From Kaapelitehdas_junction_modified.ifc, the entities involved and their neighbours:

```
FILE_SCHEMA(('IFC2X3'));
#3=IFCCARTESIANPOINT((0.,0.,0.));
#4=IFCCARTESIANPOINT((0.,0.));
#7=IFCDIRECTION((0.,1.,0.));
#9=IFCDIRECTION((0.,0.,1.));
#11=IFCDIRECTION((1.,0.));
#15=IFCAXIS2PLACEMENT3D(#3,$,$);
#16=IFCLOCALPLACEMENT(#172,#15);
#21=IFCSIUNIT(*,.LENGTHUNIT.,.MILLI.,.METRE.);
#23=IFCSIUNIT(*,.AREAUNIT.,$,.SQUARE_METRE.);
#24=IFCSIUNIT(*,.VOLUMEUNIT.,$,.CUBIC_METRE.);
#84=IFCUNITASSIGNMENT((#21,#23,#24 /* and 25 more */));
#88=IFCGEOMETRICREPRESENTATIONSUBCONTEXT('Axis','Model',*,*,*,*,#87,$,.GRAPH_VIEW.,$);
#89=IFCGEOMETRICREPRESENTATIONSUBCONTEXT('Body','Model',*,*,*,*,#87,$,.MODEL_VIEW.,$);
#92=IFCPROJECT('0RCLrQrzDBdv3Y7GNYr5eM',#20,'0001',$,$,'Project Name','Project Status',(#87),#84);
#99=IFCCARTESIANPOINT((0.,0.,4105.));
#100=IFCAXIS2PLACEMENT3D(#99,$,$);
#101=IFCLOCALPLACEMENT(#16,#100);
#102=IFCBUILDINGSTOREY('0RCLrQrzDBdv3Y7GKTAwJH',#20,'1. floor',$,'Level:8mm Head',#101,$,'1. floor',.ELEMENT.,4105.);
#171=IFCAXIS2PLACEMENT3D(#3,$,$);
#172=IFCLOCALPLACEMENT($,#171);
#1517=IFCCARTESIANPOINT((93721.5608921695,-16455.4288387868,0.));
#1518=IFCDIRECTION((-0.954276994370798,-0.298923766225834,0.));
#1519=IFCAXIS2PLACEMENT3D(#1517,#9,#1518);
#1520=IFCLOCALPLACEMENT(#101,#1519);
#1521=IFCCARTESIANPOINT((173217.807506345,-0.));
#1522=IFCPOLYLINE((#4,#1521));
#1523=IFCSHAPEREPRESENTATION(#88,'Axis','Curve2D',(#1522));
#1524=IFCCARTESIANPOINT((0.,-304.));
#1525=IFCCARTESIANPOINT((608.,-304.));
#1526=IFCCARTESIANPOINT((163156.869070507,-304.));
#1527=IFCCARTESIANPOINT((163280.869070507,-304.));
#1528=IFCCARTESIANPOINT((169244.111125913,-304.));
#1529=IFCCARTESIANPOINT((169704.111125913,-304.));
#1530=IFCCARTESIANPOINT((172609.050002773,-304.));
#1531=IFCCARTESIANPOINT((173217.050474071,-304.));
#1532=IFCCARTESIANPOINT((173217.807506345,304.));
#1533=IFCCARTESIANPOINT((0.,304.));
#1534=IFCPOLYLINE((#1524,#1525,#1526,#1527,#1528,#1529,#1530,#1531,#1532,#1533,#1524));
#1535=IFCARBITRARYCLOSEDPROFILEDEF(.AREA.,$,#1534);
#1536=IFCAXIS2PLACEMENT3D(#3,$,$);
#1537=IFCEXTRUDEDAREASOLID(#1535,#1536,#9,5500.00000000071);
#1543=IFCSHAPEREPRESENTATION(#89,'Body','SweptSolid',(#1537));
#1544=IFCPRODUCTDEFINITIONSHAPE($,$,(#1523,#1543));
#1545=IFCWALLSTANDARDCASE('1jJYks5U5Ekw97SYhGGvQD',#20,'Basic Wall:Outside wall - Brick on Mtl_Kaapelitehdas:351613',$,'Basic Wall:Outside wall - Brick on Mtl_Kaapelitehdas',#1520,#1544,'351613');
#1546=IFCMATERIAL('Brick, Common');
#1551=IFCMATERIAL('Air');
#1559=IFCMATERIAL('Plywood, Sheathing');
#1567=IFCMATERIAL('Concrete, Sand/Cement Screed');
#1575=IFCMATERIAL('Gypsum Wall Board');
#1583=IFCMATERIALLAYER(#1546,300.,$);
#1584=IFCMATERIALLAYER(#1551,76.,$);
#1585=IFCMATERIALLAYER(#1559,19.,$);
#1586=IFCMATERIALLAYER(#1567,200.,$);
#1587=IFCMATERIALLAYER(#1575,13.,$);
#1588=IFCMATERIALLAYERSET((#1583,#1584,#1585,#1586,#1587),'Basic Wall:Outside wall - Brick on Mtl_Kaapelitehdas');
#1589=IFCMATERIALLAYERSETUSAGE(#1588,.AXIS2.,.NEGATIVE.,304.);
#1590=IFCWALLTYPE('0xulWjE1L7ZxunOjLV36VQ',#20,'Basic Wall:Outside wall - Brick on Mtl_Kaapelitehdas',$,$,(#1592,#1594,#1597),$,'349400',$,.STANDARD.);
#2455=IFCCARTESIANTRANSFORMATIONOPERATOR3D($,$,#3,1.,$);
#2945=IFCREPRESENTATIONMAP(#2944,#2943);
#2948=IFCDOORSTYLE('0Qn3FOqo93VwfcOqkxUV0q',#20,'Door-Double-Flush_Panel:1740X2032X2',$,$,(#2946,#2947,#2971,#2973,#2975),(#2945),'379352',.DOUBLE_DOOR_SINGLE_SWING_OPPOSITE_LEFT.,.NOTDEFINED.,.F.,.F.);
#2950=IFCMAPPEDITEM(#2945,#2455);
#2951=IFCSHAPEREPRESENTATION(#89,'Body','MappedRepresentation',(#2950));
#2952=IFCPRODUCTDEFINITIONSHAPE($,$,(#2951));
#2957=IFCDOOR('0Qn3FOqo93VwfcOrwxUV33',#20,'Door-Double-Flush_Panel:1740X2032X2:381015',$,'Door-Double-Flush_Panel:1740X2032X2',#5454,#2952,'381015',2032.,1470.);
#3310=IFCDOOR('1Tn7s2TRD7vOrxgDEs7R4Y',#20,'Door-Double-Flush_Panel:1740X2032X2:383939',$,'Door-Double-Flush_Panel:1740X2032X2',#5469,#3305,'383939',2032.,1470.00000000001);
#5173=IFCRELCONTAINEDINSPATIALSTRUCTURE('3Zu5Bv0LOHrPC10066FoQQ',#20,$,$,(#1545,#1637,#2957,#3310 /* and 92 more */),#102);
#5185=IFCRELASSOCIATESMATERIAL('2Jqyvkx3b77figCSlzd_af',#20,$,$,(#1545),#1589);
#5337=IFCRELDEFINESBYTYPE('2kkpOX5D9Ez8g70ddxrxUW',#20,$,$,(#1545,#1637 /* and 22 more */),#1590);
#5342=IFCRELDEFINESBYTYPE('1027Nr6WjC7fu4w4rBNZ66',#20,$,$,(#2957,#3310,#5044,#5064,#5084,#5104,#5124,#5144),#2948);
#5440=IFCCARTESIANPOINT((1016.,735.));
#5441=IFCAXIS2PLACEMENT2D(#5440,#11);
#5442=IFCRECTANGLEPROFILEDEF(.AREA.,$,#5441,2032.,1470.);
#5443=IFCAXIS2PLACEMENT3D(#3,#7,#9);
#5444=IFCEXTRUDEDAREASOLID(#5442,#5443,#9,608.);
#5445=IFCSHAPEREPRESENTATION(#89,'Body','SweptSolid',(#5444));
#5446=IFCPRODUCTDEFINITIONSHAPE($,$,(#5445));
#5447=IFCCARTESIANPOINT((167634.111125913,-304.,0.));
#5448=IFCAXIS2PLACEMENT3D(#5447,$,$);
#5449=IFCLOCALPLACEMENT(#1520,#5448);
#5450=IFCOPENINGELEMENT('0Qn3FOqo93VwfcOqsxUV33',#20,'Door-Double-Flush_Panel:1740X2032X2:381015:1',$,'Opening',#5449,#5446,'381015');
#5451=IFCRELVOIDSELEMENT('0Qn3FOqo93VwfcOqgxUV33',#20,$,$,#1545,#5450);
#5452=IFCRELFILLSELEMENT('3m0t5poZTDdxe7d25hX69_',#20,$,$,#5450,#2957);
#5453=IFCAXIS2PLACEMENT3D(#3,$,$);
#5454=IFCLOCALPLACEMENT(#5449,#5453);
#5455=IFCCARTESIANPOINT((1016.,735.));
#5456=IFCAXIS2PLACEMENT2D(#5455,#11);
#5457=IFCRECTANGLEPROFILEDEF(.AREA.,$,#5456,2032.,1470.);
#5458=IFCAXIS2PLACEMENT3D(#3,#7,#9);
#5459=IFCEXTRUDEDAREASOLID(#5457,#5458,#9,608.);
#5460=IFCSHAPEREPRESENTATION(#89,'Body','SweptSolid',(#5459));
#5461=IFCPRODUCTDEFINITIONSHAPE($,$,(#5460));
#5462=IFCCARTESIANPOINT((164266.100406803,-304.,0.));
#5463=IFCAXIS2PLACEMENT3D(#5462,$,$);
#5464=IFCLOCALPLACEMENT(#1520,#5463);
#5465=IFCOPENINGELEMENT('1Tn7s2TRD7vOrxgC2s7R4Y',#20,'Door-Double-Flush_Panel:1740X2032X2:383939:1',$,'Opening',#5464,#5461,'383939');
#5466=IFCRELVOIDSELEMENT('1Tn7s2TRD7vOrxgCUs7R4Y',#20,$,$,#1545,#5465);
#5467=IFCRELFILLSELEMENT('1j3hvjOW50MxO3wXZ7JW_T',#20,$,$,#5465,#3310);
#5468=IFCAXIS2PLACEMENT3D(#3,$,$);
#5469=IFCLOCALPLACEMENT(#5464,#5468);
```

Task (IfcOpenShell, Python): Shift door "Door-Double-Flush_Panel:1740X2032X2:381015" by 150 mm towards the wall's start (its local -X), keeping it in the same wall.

```python
import ifcopenshell
import ifcopenshell.api.geometry
import ifcopenshell.util.placement

model = ifcopenshell.open("Kaapelitehdas_junction_modified.ifc")

door = model.by_guid("0Qn3FOqo93VwfcOrwxUV33")
opening = door.FillsVoids[0].RelatingOpeningElement
wall = opening.VoidsElements[0].RelatingBuildingElement

wall_matrix = ifcopenshell.util.placement.get_local_placement(wall.ObjectPlacement)
shift = wall_matrix[:3, 0] * -150.0
before = ifcopenshell.util.placement.get_local_placement(door.ObjectPlacement)[:3, 3].copy()

# The door is placed relative to its opening, so it follows when the opening moves.
matrix = ifcopenshell.util.placement.get_local_placement(opening.ObjectPlacement)
matrix[:3, 3] += shift
ifcopenshell.api.geometry.edit_object_placement(
    model, product=opening, matrix=matrix, is_si=False, should_transform_children=True
)

after = ifcopenshell.util.placement.get_local_placement(door.ObjectPlacement)[:3, 3]
print("door moved by", (after - before).round(3) + 0.0)

model.write("Kaapelitehdas_junction_modified_edited.ifc")
```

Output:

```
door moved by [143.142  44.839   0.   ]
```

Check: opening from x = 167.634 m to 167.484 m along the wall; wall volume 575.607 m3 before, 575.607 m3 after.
